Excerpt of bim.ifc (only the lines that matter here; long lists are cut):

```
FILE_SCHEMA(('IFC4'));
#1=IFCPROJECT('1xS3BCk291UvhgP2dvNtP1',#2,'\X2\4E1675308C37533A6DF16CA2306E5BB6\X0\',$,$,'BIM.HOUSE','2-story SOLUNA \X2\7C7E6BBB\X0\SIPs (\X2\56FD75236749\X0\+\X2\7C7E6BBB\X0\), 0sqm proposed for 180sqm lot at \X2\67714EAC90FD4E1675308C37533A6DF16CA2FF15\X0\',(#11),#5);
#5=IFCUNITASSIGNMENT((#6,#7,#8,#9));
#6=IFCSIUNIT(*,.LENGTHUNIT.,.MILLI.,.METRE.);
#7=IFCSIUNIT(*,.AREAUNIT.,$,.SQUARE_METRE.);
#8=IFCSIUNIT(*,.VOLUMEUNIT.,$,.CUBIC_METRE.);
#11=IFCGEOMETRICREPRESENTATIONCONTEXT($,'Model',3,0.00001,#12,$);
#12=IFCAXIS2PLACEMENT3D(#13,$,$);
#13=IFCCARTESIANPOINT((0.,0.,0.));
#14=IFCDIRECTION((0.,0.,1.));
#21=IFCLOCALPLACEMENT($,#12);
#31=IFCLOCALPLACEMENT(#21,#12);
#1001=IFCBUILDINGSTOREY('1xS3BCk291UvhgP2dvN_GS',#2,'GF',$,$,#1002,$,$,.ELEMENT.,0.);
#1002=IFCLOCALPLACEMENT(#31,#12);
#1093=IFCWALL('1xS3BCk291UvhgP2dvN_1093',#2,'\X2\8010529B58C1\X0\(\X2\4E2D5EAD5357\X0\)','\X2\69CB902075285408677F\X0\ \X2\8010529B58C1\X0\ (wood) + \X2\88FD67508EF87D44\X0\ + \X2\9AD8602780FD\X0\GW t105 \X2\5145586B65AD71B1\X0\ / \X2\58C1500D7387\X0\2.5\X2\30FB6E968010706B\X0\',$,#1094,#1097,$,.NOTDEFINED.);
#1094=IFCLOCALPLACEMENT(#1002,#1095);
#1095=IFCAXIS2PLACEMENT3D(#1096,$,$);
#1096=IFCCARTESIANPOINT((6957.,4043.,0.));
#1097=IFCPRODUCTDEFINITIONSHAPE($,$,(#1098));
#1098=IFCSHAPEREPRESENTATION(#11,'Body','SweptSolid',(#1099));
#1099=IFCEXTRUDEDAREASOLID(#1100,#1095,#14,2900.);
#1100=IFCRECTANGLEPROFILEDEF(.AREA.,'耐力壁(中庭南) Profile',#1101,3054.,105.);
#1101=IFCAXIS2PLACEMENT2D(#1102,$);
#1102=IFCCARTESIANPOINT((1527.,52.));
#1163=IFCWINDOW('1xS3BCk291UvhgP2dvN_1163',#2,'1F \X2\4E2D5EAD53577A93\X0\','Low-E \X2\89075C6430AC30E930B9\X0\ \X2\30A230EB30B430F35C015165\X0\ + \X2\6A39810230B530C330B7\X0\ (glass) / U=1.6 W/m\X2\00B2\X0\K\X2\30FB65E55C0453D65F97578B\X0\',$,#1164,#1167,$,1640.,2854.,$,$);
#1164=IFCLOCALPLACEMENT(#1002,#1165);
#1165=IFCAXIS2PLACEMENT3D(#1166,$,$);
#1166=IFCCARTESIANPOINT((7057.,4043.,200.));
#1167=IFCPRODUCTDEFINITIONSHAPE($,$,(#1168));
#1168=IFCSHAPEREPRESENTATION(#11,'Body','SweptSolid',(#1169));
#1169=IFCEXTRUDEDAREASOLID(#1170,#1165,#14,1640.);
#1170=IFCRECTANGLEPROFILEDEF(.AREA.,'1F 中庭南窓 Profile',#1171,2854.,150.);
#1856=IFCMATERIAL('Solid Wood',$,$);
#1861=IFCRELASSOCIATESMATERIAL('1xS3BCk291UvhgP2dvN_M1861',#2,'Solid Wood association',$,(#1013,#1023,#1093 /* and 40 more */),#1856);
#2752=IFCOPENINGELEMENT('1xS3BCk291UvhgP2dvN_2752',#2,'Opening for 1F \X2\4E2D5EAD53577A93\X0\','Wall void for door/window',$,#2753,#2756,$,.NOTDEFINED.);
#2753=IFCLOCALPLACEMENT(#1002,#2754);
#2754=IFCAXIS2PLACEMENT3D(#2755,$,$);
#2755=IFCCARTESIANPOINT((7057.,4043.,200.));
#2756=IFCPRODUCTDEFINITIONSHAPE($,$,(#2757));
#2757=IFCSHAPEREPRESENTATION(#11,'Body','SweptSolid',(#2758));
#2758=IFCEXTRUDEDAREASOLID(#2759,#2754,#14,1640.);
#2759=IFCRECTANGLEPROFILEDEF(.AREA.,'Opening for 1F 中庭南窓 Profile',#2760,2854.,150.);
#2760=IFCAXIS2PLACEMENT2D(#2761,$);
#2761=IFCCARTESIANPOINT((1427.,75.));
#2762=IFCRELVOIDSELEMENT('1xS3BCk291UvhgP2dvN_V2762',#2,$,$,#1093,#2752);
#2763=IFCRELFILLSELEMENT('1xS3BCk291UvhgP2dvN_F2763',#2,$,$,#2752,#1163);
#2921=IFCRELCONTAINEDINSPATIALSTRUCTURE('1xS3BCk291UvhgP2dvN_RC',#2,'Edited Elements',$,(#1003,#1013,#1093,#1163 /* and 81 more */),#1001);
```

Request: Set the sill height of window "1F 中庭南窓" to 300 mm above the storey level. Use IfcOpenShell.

```python
import numpy as np
import ifcopenshell
import ifcopenshell.api.geometry
import ifcopenshell.geom
import ifcopenshell.util.element
import ifcopenshell.util.placement
import ifcopenshell.util.shape
import ifcopenshell.util.unit

model = ifcopenshell.open("bim.ifc")
unit_scale = ifcopenshell.util.unit.calculate_unit_scale(model)

window = model.by_id(1163)
opening = window.FillsVoids[0].RelatingOpeningElement
storey = ifcopenshell.util.element.get_container(window, ifc_class="IfcBuildingStorey")
level = ifcopenshell.util.placement.get_local_placement(storey.ObjectPlacement)[2, 3]

# The opening's origin need not be at the sill, so measure its lowest point.
shape = ifcopenshell.geom.create_shape(ifcopenshell.geom.settings(), opening)
bottom = ifcopenshell.util.shape.get_shape_bottom_elevation(shape, shape.geometry) / unit_scale
dz = level + 0.3 / unit_scale - bottom

shift = np.array([0.0, 0.0, dz])
# The window is not placed relative to its opening, so move both.
for product in (opening, window):
    matrix = ifcopenshell.util.placement.get_local_placement(product.ObjectPlacement)
    matrix[:3, 3] += shift
    ifcopenshell.api.geometry.edit_object_placement(model, product=product, matrix=matrix, is_si=False)

print(f"moved by {dz * unit_scale:+.3f} m")

model.write("bim-out.ifc")
```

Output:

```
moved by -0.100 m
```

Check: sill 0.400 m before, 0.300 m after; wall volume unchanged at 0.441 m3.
